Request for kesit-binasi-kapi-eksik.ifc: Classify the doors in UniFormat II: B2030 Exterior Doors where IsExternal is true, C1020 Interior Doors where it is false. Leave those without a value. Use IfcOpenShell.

First a look at what the model holds.

```python
import ifcopenshell
import ifcopenshell.util.element

model = ifcopenshell.open("kesit-binasi-kapi-eksik.ifc")
print(model.schema)
print("classifications:", [c.Name for c in model.by_type("IfcClassification")])
values = [ifcopenshell.util.element.get_pset(e, "Pset_DoorCommon", "IsExternal") for e in model.by_type("IfcDoor")]
for value in (True, False, None):
    print("IsExternal", value, values.count(value))
```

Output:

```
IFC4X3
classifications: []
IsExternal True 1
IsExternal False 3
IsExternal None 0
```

```python
import ifcopenshell
import ifcopenshell.api.classification
import ifcopenshell.util.element

model = ifcopenshell.open("kesit-binasi-kapi-eksik.ifc")

system = ifcopenshell.api.classification.add_classification(model, classification="UniFormat II")

doors = model.by_type("IfcDoor")
external = {e: ifcopenshell.util.element.get_pset(e, "Pset_DoorCommon", "IsExternal") for e in doors}
for flag, code, name in ((True, "B2030", "Exterior Doors"), (False, "C1020", "Interior Doors")):
    products = [e for e in doors if external[e] is flag]
    ifcopenshell.api.classification.add_reference(
        model, products=products, classification=system, identification=code, name=name
    )
    print(code, len(products))

model.write("kesit-binasi-kapi-eksik_rev.ifc")
```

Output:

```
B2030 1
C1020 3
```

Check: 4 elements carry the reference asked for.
